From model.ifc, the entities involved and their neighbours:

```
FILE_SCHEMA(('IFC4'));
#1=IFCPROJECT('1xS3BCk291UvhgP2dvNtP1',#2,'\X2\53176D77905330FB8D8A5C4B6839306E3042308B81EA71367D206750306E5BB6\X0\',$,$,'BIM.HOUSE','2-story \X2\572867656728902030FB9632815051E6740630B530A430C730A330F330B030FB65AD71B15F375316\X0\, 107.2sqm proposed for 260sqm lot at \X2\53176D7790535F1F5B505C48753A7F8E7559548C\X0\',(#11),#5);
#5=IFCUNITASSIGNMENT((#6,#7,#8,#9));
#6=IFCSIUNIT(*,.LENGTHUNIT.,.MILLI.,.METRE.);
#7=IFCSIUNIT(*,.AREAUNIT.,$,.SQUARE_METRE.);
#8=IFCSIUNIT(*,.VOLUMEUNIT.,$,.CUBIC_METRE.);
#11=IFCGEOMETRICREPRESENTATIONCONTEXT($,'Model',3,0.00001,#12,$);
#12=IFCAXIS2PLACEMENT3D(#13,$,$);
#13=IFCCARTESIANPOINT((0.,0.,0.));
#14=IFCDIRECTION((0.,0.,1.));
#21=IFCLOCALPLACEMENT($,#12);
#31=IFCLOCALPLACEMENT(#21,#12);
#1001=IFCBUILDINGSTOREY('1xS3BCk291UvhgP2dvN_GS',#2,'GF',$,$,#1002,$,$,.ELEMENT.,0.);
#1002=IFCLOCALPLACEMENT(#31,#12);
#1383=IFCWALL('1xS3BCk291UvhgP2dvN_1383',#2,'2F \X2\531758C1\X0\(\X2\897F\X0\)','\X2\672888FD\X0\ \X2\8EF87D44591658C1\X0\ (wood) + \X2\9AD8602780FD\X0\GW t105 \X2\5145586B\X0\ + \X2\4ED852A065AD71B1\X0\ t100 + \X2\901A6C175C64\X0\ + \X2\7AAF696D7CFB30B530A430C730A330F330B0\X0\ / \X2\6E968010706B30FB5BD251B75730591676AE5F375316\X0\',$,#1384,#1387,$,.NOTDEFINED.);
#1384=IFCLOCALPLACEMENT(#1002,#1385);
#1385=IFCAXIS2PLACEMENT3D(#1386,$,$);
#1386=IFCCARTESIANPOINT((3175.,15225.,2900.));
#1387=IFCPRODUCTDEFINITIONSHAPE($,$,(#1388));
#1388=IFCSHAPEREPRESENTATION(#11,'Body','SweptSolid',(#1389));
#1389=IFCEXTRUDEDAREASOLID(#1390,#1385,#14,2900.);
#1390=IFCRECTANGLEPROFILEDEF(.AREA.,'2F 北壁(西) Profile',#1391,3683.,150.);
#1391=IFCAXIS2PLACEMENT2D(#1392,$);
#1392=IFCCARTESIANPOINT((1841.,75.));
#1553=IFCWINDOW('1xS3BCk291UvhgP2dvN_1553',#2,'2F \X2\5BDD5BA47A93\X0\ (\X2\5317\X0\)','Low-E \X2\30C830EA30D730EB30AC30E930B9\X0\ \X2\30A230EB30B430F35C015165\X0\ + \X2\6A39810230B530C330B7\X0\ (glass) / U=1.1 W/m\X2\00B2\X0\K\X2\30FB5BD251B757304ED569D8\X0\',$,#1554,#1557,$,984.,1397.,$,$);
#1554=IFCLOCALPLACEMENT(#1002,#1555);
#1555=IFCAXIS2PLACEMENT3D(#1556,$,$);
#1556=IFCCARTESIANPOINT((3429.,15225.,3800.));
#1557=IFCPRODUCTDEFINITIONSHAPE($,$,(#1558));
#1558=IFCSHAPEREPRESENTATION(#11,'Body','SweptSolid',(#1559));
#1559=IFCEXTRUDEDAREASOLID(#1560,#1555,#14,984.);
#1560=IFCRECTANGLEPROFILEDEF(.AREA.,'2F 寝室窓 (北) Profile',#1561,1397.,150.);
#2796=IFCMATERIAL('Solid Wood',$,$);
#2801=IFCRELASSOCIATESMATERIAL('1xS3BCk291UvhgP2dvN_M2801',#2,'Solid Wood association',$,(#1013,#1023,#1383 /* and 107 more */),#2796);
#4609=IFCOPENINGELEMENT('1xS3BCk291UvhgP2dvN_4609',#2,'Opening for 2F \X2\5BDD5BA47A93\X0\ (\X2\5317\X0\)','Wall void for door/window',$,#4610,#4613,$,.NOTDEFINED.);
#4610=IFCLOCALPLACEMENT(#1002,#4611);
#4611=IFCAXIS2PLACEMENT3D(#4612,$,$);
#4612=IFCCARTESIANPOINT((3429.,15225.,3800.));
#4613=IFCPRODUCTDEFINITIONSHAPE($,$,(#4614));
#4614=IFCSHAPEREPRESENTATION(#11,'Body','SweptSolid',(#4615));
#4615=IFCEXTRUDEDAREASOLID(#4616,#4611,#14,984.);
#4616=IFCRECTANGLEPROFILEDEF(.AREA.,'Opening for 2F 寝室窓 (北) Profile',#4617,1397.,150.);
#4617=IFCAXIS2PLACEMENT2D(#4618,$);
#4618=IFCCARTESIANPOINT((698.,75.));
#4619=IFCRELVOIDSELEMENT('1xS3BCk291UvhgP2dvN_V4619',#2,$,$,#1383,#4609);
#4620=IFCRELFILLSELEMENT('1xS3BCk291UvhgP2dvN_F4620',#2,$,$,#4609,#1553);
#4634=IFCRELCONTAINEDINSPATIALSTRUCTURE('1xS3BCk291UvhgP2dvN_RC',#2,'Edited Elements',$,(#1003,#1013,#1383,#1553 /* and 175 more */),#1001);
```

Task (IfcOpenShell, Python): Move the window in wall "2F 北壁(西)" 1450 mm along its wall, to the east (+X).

```python
import ifcopenshell
import ifcopenshell.api.geometry
import ifcopenshell.util.placement

model = ifcopenshell.open("model.ifc")

window = model.by_id(1553)
opening = window.FillsVoids[0].RelatingOpeningElement
wall = opening.VoidsElements[0].RelatingBuildingElement

wall_matrix = ifcopenshell.util.placement.get_local_placement(wall.ObjectPlacement)
shift = wall_matrix[:3, 0] * 1450.0
before = ifcopenshell.util.placement.get_local_placement(window.ObjectPlacement)[:3, 3].copy()

# The window is not placed relative to its opening, so move both.
for product in (opening, window):
    matrix = ifcopenshell.util.placement.get_local_placement(product.ObjectPlacement)
    matrix[:3, 3] += shift
    ifcopenshell.api.geometry.edit_object_placement(model, product=product, matrix=matrix, is_si=False)

after = ifcopenshell.util.placement.get_local_placement(window.ObjectPlacement)[:3, 3]
print("window moved by", (after - before).round(3) + 0.0)

model.write("model_updated.ifc")
```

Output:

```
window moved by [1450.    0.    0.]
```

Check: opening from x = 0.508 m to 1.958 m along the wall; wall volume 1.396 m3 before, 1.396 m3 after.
